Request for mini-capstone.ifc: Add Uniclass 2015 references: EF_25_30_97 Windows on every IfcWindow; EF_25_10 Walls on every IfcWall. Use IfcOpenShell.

First a look at what the model holds.

```python
import ifcopenshell

model = ifcopenshell.open("mini-capstone.ifc")
print(model.schema)
print("classifications:", [c.Name for c in model.by_type("IfcClassification")])
for ifc_class in ("IfcDoor", "IfcRoof", "IfcStair", "IfcWall", "IfcWindow"):
    print(ifc_class, len(model.by_type(ifc_class)))
```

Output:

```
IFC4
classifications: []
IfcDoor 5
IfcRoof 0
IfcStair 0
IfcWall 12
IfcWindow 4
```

```python
import ifcopenshell
import ifcopenshell.api.classification

model = ifcopenshell.open("mini-capstone.ifc")

system = ifcopenshell.api.classification.add_classification(model, classification="Uniclass 2015")

codes = {
    "IfcWindow": ("EF_25_30_97", "Windows"),
    "IfcWall": ("EF_25_10", "Walls"),
}
for ifc_class, (code, name) in codes.items():
    products = model.by_type(ifc_class)
    ifcopenshell.api.classification.add_reference(
        model, products=products, classification=system, identification=code, name=name
    )
    print(code, len(products))

model.write("mini-capstone_edited.ifc")
```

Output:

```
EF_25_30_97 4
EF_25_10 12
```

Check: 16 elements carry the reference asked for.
